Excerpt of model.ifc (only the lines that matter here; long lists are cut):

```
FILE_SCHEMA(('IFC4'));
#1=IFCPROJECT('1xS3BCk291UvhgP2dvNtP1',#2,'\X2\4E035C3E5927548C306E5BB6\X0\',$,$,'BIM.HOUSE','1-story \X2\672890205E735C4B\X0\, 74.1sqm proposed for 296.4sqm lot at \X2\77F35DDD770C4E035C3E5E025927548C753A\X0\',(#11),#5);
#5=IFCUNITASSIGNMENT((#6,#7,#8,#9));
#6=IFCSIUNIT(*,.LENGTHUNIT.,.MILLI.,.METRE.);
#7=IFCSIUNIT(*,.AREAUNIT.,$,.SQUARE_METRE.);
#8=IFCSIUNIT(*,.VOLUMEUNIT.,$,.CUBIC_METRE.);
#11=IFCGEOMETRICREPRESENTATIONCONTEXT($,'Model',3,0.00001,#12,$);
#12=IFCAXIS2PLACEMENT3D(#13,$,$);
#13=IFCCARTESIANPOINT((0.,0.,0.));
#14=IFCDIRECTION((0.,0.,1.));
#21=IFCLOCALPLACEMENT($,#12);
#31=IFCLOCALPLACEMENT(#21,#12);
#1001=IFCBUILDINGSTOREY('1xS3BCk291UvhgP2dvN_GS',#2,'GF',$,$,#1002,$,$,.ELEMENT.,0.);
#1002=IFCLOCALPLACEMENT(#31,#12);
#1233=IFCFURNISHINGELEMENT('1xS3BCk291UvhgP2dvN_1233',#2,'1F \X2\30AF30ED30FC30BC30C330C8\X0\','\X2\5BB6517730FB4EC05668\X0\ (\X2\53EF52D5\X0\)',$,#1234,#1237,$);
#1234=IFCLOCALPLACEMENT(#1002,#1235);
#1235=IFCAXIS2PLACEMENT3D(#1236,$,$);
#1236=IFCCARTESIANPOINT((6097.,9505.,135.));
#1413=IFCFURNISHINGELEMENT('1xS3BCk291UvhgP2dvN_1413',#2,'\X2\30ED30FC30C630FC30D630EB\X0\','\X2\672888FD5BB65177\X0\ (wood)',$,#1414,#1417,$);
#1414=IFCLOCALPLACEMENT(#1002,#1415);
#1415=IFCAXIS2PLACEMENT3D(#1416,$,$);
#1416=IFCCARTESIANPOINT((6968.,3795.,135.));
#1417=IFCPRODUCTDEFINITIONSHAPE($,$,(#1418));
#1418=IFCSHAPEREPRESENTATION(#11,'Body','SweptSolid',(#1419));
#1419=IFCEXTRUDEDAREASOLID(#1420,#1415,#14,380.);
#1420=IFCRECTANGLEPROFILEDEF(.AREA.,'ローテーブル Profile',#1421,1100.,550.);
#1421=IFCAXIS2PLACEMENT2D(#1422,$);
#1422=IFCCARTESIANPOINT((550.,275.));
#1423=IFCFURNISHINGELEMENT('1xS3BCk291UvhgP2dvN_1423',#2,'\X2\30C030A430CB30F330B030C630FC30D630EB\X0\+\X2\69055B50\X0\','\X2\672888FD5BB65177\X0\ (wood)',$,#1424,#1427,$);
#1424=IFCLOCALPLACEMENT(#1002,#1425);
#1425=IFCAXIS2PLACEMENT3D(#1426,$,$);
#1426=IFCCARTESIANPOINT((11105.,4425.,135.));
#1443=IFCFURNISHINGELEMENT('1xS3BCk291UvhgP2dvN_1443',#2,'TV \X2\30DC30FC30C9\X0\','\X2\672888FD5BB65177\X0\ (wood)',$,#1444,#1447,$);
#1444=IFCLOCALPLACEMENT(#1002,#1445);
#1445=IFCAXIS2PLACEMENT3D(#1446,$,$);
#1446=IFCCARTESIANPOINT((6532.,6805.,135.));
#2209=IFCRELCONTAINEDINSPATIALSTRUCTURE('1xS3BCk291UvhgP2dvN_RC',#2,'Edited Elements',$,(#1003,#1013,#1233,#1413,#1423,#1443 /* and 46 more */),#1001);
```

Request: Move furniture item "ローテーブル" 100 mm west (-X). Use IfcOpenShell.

```python
import ifcopenshell
import ifcopenshell.api.geometry
import ifcopenshell.util.placement

model = ifcopenshell.open("model.ifc")

item = model.by_guid("1xS3BCk291UvhgP2dvN_1413")
matrix = ifcopenshell.util.placement.get_local_placement(item.ObjectPlacement)
matrix[0, 3] -= 100.0
ifcopenshell.api.geometry.edit_object_placement(model, product=item, matrix=matrix, is_si=False)

print(ifcopenshell.util.placement.get_local_placement(item.ObjectPlacement).round(3) + 0.0)

model.write("model_v2.ifc")
```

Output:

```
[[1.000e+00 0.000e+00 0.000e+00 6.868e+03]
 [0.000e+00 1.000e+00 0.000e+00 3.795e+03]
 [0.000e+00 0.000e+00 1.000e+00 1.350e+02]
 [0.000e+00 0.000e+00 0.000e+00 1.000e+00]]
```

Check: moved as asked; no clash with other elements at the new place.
